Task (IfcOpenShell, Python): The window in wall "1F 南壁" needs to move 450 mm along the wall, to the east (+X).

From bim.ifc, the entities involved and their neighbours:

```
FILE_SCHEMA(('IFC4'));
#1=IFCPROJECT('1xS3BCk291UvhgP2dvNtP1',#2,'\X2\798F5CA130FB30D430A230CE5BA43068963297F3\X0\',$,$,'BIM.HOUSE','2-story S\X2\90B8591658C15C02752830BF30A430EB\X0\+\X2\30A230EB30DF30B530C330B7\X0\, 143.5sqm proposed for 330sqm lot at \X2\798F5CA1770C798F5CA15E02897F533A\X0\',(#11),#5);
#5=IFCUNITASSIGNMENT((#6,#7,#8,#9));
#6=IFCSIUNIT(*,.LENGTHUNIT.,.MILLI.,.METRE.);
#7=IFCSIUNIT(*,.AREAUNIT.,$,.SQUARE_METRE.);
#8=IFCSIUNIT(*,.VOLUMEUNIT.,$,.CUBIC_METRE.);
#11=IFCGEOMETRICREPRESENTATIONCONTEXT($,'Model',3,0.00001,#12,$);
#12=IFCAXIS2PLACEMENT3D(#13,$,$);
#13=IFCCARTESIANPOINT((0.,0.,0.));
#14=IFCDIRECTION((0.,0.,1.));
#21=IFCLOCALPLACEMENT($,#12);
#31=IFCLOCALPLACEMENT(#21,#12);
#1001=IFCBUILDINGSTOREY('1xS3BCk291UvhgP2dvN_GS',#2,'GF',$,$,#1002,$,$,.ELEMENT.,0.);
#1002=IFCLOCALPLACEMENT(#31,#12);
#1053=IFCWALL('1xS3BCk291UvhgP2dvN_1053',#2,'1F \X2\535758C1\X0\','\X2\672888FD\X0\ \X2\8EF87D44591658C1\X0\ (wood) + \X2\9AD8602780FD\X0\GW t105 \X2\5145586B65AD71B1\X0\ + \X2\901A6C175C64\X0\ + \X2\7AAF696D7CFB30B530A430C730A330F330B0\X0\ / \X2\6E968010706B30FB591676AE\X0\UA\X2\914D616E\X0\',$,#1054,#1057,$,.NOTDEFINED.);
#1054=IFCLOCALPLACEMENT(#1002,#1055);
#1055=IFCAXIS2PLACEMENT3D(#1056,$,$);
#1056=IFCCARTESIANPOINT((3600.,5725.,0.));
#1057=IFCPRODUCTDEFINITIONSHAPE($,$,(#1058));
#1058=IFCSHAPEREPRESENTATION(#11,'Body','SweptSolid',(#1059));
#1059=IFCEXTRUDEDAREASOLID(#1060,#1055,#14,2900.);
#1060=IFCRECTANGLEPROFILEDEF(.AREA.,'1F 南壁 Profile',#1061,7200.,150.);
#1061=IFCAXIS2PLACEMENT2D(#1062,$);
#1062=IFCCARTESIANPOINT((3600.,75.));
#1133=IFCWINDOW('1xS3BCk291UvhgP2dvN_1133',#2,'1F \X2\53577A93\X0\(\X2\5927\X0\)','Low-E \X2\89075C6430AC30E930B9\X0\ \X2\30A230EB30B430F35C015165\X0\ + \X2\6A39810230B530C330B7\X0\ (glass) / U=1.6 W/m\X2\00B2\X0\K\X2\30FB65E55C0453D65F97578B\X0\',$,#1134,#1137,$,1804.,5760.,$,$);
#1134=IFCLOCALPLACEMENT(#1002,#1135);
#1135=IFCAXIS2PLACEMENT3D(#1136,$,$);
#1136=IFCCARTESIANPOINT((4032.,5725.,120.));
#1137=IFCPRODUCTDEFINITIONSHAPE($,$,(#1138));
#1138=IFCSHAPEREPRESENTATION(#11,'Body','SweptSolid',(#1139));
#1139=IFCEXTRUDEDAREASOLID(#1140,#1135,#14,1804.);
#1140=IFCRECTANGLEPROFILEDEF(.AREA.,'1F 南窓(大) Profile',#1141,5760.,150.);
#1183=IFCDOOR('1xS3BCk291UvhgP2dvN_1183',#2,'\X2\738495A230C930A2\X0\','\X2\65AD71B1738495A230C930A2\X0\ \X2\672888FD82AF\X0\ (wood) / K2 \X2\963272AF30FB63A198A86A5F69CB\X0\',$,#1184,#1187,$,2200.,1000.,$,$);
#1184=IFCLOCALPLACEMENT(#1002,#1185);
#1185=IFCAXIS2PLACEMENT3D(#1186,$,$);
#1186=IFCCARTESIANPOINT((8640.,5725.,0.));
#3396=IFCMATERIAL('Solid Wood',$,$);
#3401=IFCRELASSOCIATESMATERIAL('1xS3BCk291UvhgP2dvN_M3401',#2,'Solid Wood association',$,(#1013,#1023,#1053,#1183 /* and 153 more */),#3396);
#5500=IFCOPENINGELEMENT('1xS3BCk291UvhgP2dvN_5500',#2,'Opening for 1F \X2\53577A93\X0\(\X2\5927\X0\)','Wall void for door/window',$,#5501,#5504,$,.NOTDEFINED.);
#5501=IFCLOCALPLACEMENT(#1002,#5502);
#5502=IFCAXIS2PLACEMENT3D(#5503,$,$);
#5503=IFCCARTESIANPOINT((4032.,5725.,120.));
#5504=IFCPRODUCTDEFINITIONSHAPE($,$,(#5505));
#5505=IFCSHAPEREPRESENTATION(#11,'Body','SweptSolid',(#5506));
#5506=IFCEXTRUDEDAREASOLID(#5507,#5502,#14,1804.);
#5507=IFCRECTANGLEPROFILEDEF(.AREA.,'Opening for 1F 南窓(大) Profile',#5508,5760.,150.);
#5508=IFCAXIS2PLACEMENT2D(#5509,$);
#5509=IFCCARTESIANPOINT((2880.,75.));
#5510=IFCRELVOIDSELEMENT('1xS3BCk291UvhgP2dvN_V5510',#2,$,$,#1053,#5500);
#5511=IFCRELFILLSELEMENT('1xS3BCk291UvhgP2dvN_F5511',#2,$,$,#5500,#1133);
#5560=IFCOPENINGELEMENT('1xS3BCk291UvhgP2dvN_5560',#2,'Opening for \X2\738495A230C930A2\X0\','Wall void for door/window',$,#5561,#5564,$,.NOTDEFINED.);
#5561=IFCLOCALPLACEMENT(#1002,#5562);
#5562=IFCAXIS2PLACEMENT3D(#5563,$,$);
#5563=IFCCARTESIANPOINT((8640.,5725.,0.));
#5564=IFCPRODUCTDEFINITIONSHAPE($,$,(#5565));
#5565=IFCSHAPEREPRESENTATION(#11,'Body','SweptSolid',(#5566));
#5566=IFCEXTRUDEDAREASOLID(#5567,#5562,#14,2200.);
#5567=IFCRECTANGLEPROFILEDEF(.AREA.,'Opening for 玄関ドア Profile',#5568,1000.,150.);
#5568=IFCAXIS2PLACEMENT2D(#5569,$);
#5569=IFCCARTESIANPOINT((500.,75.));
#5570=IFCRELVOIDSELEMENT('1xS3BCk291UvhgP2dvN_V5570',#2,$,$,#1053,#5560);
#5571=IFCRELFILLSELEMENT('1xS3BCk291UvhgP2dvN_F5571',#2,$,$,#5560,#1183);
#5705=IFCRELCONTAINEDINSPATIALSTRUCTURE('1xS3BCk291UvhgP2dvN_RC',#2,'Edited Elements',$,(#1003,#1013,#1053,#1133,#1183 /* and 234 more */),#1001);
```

```python
import ifcopenshell
import ifcopenshell.api.geometry
import ifcopenshell.util.placement
import ifcopenshell.util.unit

model = ifcopenshell.open("bim.ifc")
unit_scale = ifcopenshell.util.unit.calculate_unit_scale(model)

window = model.by_guid("1xS3BCk291UvhgP2dvN_1133")
opening = window.FillsVoids[0].RelatingOpeningElement
wall = opening.VoidsElements[0].RelatingBuildingElement

wall_matrix = ifcopenshell.util.placement.get_local_placement(wall.ObjectPlacement)
shift = wall_matrix[:3, 0] * 0.45 / unit_scale
before = ifcopenshell.util.placement.get_local_placement(window.ObjectPlacement)[:3, 3].copy()

# The window is not placed relative to its opening, so move both.
for product in (opening, window):
    matrix = ifcopenshell.util.placement.get_local_placement(product.ObjectPlacement)
    matrix[:3, 3] += shift
    ifcopenshell.api.geometry.edit_object_placement(model, product=product, matrix=matrix, is_si=False)

after = ifcopenshell.util.placement.get_local_placement(window.ObjectPlacement)[:3, 3]
print("window moved by", (after - before).round(3) + 0.0)

model.write("bim_updated.ifc")
```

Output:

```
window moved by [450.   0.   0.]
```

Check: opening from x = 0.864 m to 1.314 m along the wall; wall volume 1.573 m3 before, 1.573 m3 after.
